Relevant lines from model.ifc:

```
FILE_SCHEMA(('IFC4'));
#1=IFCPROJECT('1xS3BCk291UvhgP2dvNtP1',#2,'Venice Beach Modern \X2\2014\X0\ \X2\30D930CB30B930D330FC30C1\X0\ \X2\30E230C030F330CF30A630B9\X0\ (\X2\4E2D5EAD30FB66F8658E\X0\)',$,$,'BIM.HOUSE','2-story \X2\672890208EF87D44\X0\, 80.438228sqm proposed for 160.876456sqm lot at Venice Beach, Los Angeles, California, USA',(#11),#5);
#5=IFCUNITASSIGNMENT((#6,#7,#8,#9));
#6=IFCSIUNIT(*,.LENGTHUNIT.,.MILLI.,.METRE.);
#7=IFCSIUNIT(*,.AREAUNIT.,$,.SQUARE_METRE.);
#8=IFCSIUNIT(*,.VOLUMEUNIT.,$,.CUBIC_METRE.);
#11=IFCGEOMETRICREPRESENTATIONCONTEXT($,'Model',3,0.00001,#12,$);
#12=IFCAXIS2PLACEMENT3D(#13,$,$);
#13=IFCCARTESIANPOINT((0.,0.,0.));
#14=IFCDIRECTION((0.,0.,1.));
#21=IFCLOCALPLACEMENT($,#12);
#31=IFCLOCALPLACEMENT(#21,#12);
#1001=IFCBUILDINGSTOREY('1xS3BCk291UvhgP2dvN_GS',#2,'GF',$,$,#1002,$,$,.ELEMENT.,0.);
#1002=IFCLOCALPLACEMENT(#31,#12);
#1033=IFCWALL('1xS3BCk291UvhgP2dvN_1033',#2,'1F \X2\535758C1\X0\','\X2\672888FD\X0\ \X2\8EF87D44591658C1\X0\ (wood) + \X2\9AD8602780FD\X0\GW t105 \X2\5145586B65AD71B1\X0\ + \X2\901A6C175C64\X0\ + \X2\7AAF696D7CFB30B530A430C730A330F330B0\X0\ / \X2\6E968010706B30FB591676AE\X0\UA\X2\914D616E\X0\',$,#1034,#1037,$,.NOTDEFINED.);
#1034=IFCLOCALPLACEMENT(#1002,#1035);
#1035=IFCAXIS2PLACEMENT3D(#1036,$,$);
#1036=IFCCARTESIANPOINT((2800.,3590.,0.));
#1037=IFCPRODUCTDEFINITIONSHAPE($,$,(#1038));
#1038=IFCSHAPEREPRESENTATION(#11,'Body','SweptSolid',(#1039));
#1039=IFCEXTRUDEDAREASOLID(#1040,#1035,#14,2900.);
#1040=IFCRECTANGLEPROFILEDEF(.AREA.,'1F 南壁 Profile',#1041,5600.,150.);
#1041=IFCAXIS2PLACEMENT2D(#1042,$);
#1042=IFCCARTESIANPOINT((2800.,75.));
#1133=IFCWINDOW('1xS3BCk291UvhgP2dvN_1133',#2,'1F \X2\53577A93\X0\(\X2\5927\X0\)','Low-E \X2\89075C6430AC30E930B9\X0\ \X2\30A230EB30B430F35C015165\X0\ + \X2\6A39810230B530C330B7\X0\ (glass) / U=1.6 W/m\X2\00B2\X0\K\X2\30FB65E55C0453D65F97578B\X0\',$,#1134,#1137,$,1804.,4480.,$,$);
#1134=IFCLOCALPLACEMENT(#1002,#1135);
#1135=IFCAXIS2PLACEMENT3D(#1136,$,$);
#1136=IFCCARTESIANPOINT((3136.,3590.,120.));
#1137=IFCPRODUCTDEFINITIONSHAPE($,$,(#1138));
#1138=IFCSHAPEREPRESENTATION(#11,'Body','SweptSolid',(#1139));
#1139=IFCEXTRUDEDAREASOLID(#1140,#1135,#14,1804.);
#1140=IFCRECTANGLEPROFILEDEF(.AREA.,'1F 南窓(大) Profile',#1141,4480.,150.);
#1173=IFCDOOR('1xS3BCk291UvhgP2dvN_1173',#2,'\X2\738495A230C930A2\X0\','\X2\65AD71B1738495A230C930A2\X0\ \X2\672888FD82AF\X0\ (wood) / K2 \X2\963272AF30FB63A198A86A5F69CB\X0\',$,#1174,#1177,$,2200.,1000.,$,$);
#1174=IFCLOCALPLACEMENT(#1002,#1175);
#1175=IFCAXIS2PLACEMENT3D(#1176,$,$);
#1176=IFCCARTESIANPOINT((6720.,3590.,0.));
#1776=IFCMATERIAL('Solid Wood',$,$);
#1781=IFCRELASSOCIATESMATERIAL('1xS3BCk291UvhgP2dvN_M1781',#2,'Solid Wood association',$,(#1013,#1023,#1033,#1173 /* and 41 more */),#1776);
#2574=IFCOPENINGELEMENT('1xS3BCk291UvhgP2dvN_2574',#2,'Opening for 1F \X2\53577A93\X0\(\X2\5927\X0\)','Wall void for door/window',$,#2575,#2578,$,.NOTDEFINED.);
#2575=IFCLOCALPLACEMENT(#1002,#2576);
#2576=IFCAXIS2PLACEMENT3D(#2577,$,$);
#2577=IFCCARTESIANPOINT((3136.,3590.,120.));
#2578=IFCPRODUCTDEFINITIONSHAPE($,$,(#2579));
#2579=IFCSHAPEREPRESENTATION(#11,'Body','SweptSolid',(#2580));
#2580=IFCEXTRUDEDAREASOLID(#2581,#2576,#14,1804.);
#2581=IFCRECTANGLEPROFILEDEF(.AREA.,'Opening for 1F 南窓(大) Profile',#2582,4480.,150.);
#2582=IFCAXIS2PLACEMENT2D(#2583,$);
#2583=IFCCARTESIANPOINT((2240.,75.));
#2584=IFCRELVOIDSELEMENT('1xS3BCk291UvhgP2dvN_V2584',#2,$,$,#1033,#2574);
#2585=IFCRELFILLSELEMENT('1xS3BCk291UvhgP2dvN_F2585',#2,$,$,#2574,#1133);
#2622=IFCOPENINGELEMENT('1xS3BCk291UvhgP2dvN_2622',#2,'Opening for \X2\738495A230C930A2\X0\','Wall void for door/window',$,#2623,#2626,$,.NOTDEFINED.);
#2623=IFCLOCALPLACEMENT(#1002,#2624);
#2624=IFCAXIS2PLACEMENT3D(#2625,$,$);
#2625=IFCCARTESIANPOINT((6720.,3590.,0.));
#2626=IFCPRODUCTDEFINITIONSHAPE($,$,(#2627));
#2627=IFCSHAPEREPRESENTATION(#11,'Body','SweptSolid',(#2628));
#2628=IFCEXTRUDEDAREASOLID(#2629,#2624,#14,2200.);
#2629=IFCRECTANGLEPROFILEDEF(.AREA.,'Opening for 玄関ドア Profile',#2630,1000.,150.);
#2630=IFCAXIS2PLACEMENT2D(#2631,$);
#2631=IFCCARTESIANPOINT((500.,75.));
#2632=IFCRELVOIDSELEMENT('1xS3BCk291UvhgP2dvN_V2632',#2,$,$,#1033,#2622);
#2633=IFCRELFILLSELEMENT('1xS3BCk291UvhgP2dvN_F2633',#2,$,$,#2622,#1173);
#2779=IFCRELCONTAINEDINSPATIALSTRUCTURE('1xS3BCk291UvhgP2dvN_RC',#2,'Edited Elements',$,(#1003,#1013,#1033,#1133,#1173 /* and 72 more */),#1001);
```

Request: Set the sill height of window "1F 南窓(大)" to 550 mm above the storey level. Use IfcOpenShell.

```python
import numpy as np
import ifcopenshell
import ifcopenshell.api.geometry
import ifcopenshell.geom
import ifcopenshell.util.element
import ifcopenshell.util.placement
import ifcopenshell.util.shape
import ifcopenshell.util.unit

model = ifcopenshell.open("model.ifc")
unit_scale = ifcopenshell.util.unit.calculate_unit_scale(model)

window = model.by_guid("1xS3BCk291UvhgP2dvN_1133")
opening = window.FillsVoids[0].RelatingOpeningElement
storey = ifcopenshell.util.element.get_container(window, ifc_class="IfcBuildingStorey")
level = ifcopenshell.util.placement.get_local_placement(storey.ObjectPlacement)[2, 3]

# The opening's origin need not be at the sill, so measure its lowest point.
shape = ifcopenshell.geom.create_shape(ifcopenshell.geom.settings(), opening)
bottom = ifcopenshell.util.shape.get_shape_bottom_elevation(shape, shape.geometry) / unit_scale
dz = level + 0.55 / unit_scale - bottom

shift = np.array([0.0, 0.0, dz])
# The window is not placed relative to its opening, so move both.
for product in (opening, window):
    matrix = ifcopenshell.util.placement.get_local_placement(product.ObjectPlacement)
    matrix[:3, 3] += shift
    ifcopenshell.api.geometry.edit_object_placement(model, product=product, matrix=matrix, is_si=False)

print(f"moved by {dz * unit_scale:+.3f} m")

model.write("model_v2.ifc")
```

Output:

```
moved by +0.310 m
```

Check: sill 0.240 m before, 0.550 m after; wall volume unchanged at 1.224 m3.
